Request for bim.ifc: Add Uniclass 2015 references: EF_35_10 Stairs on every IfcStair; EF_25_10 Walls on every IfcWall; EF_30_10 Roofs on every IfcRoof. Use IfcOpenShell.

First a look at what the model holds.

```python
import ifcopenshell

model = ifcopenshell.open("bim.ifc")
print(model.schema)
print("classifications:", [c.Name for c in model.by_type("IfcClassification")])
for ifc_class in ("IfcDoor", "IfcRoof", "IfcStair", "IfcWall", "IfcWindow"):
    print(ifc_class, len(model.by_type(ifc_class)))
```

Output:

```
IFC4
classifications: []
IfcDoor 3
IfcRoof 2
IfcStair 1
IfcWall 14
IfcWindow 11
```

```python
import ifcopenshell
import ifcopenshell.api.classification

model = ifcopenshell.open("bim.ifc")

system = ifcopenshell.api.classification.add_classification(model, classification="Uniclass 2015")

codes = {
    "IfcStair": ("EF_35_10", "Stairs"),
    "IfcWall": ("EF_25_10", "Walls"),
    "IfcRoof": ("EF_30_10", "Roofs"),
}
for ifc_class, (code, name) in codes.items():
    products = model.by_type(ifc_class)
    ifcopenshell.api.classification.add_reference(
        model, products=products, classification=system, identification=code, name=name
    )
    print(code, len(products))

model.write("bim_v2.ifc")
```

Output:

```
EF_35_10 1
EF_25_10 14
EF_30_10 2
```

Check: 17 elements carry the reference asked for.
